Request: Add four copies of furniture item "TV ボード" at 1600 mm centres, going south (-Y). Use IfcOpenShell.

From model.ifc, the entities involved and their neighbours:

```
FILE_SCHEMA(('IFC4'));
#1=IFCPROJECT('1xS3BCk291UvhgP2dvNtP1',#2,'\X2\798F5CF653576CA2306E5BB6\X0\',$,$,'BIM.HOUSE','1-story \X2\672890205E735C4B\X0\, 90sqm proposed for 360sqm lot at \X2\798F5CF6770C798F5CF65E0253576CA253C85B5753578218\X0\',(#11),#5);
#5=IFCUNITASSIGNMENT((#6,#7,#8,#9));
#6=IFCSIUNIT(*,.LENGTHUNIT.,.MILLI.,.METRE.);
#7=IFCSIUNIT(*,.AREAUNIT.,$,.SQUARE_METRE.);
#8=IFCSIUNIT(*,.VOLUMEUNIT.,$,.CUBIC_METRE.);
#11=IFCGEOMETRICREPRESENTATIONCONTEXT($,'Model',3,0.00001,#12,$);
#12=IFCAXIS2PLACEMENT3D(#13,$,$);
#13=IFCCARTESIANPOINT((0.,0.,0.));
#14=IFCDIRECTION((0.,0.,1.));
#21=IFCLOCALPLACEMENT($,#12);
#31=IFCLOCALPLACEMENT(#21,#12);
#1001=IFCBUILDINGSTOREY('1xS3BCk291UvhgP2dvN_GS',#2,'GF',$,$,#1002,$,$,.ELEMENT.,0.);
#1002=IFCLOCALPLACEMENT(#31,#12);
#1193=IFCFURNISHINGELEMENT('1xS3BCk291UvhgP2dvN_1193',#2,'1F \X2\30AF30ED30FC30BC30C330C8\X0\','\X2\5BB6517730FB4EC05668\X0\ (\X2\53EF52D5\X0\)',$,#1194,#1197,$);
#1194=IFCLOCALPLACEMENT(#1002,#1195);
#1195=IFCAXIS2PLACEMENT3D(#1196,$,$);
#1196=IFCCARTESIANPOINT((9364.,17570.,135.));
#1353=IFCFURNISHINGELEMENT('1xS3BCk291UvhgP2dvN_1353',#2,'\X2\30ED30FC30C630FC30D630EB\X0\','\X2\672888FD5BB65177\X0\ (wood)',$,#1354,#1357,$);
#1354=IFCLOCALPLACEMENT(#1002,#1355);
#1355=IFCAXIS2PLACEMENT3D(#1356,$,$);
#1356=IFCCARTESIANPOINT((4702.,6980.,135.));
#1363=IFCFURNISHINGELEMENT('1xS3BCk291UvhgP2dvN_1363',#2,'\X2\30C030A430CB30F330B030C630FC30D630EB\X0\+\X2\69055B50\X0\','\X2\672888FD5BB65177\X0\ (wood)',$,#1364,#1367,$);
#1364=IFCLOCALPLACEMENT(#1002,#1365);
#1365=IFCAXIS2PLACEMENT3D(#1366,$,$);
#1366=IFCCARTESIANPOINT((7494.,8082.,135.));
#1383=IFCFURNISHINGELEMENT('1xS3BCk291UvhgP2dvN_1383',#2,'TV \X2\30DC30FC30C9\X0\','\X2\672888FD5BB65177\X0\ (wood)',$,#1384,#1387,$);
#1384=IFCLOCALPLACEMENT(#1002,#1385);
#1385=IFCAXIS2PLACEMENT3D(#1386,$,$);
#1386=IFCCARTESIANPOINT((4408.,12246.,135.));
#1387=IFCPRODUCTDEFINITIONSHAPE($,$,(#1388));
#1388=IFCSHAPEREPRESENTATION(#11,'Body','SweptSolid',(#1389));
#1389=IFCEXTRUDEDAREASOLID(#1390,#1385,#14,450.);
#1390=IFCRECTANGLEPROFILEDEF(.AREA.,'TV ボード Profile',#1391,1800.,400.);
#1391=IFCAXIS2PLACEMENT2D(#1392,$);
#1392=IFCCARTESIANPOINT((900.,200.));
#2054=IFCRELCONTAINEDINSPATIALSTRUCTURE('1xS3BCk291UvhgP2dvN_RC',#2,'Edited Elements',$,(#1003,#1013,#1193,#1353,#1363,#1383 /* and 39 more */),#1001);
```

```python
import numpy as np
import ifcopenshell
import ifcopenshell.api.geometry
import ifcopenshell.api.root
import ifcopenshell.util.element
import ifcopenshell.util.placement

model = ifcopenshell.open("model.ifc")


def reuse_history(source, copy):
    """copy_class also copies each property set's owner history, people and application; keep the originals."""
    for rel in copy.IsDefinedBy:
        if rel.is_a("IfcRelDefinesByProperties") and (history := rel.RelatingPropertyDefinition.OwnerHistory):
            rel.RelatingPropertyDefinition.OwnerHistory = source.OwnerHistory
            ifcopenshell.util.element.remove_deep2(model, history)


source = model.by_guid("1xS3BCk291UvhgP2dvN_1383")
base = ifcopenshell.util.placement.get_local_placement(source.ObjectPlacement)
step = np.array([0.0, -1.0, 0.0]) * 1600.0

for i in range(1, 5):
    copy = ifcopenshell.api.root.copy_class(model, product=source)
    copy.Representation = ifcopenshell.util.element.copy_deep(
        model, source.Representation, exclude=["IfcGeometricRepresentationContext", "IfcRepresentationMap"]
    )
    reuse_history(source, copy)
    matrix = base.copy()
    matrix[:3, 3] += i * step
    print("added at", matrix[:3, 3].round(3) + 0.0)
    ifcopenshell.api.geometry.edit_object_placement(model, product=copy, matrix=matrix, is_si=False)

model.write("model_edited.ifc")
```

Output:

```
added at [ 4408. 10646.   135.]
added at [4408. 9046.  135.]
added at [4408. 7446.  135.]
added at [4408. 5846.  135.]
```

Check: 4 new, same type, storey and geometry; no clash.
